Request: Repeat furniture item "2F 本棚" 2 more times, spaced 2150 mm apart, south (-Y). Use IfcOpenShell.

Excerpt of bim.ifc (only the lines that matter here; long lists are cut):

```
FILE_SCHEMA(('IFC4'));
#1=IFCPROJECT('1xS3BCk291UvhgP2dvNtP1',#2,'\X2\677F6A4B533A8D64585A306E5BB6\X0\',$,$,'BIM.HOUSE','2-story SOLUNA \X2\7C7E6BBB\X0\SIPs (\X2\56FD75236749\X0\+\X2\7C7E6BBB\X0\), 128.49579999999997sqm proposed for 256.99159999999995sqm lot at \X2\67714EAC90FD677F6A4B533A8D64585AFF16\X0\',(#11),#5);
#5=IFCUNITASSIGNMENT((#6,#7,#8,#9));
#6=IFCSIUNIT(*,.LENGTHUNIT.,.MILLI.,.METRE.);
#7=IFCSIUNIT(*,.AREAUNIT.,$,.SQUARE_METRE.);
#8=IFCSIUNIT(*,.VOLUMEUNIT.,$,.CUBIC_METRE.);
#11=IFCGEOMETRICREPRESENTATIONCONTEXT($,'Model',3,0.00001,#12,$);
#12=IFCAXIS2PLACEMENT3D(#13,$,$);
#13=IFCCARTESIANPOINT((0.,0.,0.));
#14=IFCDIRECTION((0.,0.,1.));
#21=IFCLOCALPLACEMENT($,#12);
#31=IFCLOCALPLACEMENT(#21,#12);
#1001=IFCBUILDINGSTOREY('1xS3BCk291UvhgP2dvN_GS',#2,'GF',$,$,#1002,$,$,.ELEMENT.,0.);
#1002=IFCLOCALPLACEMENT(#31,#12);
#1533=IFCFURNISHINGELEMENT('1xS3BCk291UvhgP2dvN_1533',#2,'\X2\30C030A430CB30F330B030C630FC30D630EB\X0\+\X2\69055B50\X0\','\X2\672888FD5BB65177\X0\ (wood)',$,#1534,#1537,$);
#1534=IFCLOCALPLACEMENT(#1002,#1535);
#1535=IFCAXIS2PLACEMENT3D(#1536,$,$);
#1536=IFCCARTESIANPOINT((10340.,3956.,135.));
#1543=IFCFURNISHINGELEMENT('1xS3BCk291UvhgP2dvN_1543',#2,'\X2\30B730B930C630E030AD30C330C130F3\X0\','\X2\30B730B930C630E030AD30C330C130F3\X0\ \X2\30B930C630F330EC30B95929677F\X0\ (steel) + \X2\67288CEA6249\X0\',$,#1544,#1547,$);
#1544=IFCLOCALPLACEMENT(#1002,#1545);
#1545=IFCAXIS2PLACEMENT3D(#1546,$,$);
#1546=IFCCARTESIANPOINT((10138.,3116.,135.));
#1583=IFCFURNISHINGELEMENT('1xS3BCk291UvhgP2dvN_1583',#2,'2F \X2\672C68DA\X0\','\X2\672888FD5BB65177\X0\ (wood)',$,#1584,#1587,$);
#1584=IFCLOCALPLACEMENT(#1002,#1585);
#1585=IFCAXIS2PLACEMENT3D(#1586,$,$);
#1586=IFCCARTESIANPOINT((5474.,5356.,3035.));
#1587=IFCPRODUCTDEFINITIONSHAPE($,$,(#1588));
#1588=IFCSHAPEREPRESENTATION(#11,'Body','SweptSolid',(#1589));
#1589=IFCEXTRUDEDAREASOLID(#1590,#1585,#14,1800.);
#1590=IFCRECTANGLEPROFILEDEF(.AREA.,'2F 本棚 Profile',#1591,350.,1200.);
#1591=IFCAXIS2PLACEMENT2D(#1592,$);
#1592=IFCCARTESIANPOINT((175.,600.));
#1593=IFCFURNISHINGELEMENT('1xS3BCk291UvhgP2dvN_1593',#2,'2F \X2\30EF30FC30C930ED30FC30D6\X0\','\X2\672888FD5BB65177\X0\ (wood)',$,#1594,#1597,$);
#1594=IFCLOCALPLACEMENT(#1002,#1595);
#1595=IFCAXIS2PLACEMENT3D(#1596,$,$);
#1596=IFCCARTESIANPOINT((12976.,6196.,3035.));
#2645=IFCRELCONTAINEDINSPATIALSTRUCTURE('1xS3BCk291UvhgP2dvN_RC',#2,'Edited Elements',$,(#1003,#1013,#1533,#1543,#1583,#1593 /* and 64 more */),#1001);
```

```python
import numpy as np
import ifcopenshell
import ifcopenshell.api.geometry
import ifcopenshell.api.root
import ifcopenshell.util.element
import ifcopenshell.util.placement
import ifcopenshell.util.unit

model = ifcopenshell.open("bim.ifc")
unit_scale = ifcopenshell.util.unit.calculate_unit_scale(model)


def reuse_history(source, copy):
    """copy_class also copies each property set's owner history, people and application; keep the originals."""
    for rel in copy.IsDefinedBy:
        if rel.is_a("IfcRelDefinesByProperties") and (history := rel.RelatingPropertyDefinition.OwnerHistory):
            rel.RelatingPropertyDefinition.OwnerHistory = source.OwnerHistory
            ifcopenshell.util.element.remove_deep2(model, history)


source = model.by_guid("1xS3BCk291UvhgP2dvN_1583")
base = ifcopenshell.util.placement.get_local_placement(source.ObjectPlacement)
step = np.array([0.0, -1.0, 0.0]) * 2.15 / unit_scale

for i in range(1, 3):
    copy = ifcopenshell.api.root.copy_class(model, product=source)
    copy.Representation = ifcopenshell.util.element.copy_deep(
        model, source.Representation, exclude=["IfcGeometricRepresentationContext", "IfcRepresentationMap"]
    )
    reuse_history(source, copy)
    matrix = base.copy()
    matrix[:3, 3] += i * step
    print("added at", matrix[:3, 3].round(3) + 0.0)
    ifcopenshell.api.geometry.edit_object_placement(model, product=copy, matrix=matrix, is_si=False)

model.write("bim_v2.ifc")
```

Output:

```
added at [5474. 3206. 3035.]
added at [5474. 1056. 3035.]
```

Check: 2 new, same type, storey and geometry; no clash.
